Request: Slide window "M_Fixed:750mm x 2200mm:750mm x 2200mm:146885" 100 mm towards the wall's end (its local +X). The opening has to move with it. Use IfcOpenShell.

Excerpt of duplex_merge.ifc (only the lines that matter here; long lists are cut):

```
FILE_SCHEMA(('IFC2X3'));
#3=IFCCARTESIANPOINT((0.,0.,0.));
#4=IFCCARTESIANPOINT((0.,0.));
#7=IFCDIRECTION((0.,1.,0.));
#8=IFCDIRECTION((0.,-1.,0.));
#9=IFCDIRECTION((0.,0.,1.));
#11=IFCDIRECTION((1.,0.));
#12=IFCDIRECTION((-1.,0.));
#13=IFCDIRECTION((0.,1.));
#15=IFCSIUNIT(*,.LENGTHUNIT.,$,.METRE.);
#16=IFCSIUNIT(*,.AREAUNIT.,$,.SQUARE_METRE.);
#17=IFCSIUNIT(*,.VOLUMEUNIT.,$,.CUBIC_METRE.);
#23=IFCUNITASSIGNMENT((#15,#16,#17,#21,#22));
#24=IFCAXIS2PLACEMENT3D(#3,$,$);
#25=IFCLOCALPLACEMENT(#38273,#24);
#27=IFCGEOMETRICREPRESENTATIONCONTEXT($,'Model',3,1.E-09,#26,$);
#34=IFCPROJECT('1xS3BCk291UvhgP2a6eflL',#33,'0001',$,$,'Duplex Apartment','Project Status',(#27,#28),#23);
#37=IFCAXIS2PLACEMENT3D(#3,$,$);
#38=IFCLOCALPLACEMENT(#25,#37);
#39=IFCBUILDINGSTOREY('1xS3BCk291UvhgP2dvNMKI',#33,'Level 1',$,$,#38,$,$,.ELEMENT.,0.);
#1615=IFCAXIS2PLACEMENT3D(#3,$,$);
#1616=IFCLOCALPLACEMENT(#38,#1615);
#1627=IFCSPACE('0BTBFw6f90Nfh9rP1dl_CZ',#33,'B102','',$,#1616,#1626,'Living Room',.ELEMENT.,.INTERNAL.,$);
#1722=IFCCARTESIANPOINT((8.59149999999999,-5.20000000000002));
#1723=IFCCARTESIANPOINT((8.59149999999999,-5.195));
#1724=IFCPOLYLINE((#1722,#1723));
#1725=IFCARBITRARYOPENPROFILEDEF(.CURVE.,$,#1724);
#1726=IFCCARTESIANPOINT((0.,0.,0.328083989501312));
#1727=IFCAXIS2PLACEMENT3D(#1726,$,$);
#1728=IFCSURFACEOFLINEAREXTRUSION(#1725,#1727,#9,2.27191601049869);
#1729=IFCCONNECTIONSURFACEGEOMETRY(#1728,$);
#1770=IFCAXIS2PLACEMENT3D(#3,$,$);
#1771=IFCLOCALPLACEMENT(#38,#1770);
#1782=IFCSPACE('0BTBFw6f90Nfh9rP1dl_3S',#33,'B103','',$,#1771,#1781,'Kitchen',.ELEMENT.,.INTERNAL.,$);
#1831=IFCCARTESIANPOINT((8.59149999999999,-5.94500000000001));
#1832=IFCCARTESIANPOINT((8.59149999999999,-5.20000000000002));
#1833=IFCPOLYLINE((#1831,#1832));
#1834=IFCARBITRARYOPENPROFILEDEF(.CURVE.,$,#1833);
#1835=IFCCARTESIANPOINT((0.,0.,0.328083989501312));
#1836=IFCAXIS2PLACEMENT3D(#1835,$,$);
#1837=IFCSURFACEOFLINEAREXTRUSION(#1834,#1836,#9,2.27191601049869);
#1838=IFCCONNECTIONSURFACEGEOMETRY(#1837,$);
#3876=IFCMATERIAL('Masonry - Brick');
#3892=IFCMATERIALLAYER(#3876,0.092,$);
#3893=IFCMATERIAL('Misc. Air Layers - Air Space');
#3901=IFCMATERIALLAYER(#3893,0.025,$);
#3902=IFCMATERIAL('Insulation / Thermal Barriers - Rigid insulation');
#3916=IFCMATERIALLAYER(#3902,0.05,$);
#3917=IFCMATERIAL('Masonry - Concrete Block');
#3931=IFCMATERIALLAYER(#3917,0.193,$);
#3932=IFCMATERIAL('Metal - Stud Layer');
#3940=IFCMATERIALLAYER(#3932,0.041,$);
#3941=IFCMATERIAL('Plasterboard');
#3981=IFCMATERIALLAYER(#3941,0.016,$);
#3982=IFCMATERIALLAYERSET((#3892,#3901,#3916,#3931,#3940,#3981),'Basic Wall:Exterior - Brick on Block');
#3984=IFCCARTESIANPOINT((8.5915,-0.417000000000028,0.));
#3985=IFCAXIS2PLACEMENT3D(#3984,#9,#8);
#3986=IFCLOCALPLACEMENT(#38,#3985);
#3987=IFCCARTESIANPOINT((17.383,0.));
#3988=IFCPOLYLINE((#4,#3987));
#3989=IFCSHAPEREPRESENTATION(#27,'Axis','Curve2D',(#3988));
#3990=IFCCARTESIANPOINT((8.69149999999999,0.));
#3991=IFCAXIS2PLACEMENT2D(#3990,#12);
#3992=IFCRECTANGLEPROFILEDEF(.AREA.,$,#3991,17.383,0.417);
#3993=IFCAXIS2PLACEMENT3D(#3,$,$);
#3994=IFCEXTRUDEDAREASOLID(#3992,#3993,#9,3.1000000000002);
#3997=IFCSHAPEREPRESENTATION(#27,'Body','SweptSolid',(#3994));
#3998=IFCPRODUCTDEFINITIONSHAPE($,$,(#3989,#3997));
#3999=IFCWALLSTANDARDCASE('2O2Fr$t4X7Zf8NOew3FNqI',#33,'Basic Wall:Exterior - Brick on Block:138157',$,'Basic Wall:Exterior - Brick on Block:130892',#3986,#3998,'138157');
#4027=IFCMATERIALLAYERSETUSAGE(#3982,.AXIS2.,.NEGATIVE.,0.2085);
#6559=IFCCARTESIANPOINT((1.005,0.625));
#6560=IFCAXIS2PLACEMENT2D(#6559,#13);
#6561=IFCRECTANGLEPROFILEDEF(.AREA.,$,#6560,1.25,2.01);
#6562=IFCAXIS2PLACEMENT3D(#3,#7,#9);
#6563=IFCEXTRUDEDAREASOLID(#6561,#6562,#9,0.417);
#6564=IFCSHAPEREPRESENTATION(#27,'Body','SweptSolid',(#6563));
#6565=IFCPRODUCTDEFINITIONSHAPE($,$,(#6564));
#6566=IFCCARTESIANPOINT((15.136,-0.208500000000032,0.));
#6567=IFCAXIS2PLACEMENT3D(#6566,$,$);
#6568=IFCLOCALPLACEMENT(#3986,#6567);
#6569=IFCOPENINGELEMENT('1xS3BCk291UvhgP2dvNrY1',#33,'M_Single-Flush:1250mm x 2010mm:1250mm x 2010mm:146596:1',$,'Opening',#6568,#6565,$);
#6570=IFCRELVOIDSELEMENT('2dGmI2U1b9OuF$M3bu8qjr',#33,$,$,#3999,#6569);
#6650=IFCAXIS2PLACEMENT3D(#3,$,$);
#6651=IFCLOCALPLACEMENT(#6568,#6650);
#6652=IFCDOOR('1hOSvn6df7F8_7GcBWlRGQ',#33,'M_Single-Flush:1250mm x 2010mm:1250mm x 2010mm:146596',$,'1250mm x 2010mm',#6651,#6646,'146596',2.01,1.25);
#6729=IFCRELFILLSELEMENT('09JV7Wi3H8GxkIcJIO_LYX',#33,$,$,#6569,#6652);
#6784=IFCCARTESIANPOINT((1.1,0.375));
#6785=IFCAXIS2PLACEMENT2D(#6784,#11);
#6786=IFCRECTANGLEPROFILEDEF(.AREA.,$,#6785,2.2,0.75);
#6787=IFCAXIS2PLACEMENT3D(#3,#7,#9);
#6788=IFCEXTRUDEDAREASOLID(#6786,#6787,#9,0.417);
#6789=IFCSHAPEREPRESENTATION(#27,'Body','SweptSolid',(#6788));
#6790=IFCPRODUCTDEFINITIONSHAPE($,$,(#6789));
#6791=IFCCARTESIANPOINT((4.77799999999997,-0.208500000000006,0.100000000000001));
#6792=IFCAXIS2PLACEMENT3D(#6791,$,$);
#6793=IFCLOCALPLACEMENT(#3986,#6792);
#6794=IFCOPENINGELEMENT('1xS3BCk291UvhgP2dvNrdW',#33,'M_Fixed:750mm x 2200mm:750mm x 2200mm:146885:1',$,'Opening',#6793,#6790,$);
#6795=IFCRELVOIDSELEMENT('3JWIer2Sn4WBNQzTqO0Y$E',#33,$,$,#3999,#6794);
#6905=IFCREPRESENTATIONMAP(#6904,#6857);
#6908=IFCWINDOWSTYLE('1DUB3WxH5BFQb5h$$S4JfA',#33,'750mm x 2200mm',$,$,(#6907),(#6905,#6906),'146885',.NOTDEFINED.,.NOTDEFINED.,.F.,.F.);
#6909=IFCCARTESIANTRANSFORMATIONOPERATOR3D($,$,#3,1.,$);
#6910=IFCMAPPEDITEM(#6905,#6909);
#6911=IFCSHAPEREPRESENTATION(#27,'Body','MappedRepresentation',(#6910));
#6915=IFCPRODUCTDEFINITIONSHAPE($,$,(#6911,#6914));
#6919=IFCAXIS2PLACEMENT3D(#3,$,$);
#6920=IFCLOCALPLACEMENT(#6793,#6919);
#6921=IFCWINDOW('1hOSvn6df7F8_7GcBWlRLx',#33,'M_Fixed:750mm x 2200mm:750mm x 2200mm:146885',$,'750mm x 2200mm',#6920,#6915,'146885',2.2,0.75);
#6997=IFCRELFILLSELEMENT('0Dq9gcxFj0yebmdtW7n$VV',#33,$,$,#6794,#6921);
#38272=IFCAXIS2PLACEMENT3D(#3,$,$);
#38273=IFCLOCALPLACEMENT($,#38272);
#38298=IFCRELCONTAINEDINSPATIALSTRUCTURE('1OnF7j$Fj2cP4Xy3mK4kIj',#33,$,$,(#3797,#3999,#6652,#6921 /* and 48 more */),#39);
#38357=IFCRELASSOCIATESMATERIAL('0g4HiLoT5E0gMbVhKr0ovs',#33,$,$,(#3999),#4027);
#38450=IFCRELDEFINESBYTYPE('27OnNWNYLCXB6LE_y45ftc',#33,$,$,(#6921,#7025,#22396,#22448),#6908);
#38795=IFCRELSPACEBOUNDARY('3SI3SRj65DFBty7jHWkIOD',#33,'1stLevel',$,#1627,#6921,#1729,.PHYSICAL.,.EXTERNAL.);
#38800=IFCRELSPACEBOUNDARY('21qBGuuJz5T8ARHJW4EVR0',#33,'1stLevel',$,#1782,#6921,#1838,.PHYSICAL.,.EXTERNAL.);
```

```python
import numpy as np
import ifcopenshell
import ifcopenshell.api.geometry
import ifcopenshell.util.placement
import ifcopenshell.util.unit

model = ifcopenshell.open("duplex_merge.ifc")
unit_scale = ifcopenshell.util.unit.calculate_unit_scale(model)

window = model.by_guid("1hOSvn6df7F8_7GcBWlRLx")
opening = window.FillsVoids[0].RelatingOpeningElement
wall = opening.VoidsElements[0].RelatingBuildingElement

wall_matrix = ifcopenshell.util.placement.get_local_placement(wall.ObjectPlacement)
shift = wall_matrix[:3, 0] * 0.1 / unit_scale
before = ifcopenshell.util.placement.get_local_placement(window.ObjectPlacement)[:3, 3].copy()

# The window is placed relative to its opening, so it follows when the opening moves.
matrix = ifcopenshell.util.placement.get_local_placement(opening.ObjectPlacement)
matrix[:3, 3] += shift
ifcopenshell.api.geometry.edit_object_placement(
    model, product=opening, matrix=matrix, is_si=False, should_transform_children=True
)

# Space boundary surfaces are stored in each space's coordinates; move them too.
for rel in window.ProvidesBoundaries:
    if not rel.ConnectionGeometry:
        continue
    surface = rel.ConnectionGeometry.SurfaceOnRelatingElement
    space_matrix = ifcopenshell.util.placement.get_local_placement(rel.RelatingSpace.ObjectPlacement)
    point = np.array(surface.Position.Location.Coordinates) + space_matrix[:3, :3].T @ shift
    surface.Position = model.createIfcAxis2Placement3D(
        model.createIfcCartesianPoint(point.tolist()), surface.Position.Axis, surface.Position.RefDirection
    )

after = ifcopenshell.util.placement.get_local_placement(window.ObjectPlacement)[:3, 3]
print("window moved by", (after - before).round(3) + 0.0)

model.write("duplex_merge_updated.ifc")
```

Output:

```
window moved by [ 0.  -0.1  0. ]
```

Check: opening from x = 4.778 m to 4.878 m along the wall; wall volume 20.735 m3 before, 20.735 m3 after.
